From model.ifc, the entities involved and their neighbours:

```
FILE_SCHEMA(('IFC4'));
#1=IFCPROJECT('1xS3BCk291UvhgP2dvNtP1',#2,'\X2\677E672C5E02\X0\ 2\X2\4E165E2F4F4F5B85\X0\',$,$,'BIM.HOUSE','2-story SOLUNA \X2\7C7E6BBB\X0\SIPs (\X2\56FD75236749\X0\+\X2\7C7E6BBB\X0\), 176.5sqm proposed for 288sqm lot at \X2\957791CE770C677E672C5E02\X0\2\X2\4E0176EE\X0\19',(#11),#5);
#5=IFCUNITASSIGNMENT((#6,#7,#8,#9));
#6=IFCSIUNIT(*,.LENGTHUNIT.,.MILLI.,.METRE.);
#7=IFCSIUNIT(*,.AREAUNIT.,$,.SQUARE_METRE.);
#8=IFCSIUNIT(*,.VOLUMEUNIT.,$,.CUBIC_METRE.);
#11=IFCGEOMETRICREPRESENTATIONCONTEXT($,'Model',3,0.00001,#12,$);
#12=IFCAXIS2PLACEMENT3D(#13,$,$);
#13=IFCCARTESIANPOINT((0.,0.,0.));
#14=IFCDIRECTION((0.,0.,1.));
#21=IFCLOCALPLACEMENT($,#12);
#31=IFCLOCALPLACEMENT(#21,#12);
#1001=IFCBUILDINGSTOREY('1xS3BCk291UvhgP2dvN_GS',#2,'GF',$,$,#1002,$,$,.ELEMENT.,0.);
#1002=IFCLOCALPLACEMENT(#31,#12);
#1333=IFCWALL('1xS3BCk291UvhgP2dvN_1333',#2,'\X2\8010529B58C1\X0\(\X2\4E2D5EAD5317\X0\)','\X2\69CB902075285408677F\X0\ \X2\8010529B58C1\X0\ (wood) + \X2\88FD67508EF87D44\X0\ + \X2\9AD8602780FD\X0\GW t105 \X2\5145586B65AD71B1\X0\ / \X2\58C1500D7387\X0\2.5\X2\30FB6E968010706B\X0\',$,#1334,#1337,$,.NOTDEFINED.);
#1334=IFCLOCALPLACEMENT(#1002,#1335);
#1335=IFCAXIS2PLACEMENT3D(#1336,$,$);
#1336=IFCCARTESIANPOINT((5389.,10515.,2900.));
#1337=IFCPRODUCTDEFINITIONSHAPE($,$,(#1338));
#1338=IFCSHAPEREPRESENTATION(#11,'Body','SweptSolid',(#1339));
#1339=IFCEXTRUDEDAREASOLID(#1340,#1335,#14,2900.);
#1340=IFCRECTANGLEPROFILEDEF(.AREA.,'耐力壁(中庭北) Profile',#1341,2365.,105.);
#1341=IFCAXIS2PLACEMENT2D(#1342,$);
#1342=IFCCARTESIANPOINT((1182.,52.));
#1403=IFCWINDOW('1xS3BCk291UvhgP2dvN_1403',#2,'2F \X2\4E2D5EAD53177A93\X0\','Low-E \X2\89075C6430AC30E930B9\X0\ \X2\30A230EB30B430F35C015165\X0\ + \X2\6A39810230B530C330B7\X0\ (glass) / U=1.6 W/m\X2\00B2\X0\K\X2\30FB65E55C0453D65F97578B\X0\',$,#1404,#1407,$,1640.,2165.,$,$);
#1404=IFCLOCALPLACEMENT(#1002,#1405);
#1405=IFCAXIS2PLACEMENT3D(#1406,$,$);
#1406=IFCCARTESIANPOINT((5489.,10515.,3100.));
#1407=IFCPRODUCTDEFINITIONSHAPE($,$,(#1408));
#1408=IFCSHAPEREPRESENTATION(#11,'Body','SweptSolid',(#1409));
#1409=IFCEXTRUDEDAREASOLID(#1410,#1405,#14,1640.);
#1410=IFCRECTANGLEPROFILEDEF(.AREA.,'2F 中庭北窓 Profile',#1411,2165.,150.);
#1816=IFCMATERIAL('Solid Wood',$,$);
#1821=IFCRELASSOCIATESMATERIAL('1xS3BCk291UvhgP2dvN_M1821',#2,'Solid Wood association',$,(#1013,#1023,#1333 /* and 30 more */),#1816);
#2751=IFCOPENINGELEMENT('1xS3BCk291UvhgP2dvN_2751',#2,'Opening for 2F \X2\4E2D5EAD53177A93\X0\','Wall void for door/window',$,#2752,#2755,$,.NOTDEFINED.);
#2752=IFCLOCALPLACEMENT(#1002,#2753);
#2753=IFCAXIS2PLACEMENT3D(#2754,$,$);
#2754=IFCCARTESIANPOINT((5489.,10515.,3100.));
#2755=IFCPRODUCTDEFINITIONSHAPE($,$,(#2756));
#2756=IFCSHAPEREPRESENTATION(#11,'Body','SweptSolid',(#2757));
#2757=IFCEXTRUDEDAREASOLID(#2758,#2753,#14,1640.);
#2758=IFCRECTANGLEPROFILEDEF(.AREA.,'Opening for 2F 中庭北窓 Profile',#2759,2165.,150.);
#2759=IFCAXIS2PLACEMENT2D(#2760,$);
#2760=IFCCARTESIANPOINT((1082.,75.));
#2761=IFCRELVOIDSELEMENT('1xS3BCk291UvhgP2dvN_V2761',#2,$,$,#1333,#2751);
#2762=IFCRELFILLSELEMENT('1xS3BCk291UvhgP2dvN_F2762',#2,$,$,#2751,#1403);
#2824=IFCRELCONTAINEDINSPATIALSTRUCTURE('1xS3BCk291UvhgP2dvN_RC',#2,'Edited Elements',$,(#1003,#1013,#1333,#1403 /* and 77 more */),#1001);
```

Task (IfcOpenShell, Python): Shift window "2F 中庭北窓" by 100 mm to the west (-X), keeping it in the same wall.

```python
import ifcopenshell
import ifcopenshell.api.geometry
import ifcopenshell.util.placement
import ifcopenshell.util.unit

model = ifcopenshell.open("model.ifc")
unit_scale = ifcopenshell.util.unit.calculate_unit_scale(model)

window = model.by_id(1403)
opening = window.FillsVoids[0].RelatingOpeningElement
wall = opening.VoidsElements[0].RelatingBuildingElement

wall_matrix = ifcopenshell.util.placement.get_local_placement(wall.ObjectPlacement)
shift = wall_matrix[:3, 0] * -0.1 / unit_scale
before = ifcopenshell.util.placement.get_local_placement(window.ObjectPlacement)[:3, 3].copy()

# The window is not placed relative to its opening, so move both.
for product in (opening, window):
    matrix = ifcopenshell.util.placement.get_local_placement(product.ObjectPlacement)
    matrix[:3, 3] += shift
    ifcopenshell.api.geometry.edit_object_placement(model, product=product, matrix=matrix, is_si=False)

after = ifcopenshell.util.placement.get_local_placement(window.ObjectPlacement)[:3, 3]
print("window moved by", (after - before).round(3) + 0.0)

model.write("model_v2.ifc")
```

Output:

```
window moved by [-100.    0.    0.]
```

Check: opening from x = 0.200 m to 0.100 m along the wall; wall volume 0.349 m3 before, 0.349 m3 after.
